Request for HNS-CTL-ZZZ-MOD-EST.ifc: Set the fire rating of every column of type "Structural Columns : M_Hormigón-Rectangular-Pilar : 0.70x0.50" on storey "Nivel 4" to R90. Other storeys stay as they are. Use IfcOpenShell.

First a look at what the model holds.

```python
import ifcopenshell
import ifcopenshell.util.element

model = ifcopenshell.open("HNS-CTL-ZZZ-MOD-EST.ifc")
print(model.schema)
storey = next(s for s in model.by_type("IfcBuildingStorey") if s.Name == "Nivel 4")
columns = [e for e in ifcopenshell.util.element.get_decomposition(storey) if e.is_a("IfcColumn")]
seen = {}
for e in columns:
    element_type = ifcopenshell.util.element.get_type(e)
    key = (element_type.Name if element_type != e and element_type else None, ifcopenshell.util.element.get_pset(e, "Pset_ColumnCommon", "FireRating"))
    seen[key] = seen.get(key, 0) + 1
for (name, value), count in sorted(seen.items(), key=str):
    print(count, "x", name, "|", value)
```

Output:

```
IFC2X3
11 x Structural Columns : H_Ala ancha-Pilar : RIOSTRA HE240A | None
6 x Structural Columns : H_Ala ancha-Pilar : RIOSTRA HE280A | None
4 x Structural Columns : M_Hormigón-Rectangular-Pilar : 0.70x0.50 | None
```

```python
import ifcopenshell
import ifcopenshell.api.pset
import ifcopenshell.util.element

model = ifcopenshell.open("HNS-CTL-ZZZ-MOD-EST.ifc")

storey = next(s for s in model.by_type("IfcBuildingStorey") if s.Name == "Nivel 4")
columns = [e for e in ifcopenshell.util.element.get_decomposition(storey) if e.is_a("IfcColumn")]

count = 0
for e in columns:
    element_type = ifcopenshell.util.element.get_type(e)
    if element_type in (None, e) or element_type.Name != "Structural Columns : M_Hormigón-Rectangular-Pilar : 0.70x0.50":
        continue
    # add_pset returns the element's existing set when there is one.
    pset = ifcopenshell.api.pset.add_pset(model, product=e, name="Pset_ColumnCommon")
    ifcopenshell.api.pset.edit_pset(model, pset=pset, properties={"FireRating": "R90"})
    count += 1

print(count, "columns updated")

model.write("HNS-CTL-ZZZ-MOD-EST_updated.ifc")
```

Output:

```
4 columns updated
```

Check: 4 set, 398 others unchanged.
